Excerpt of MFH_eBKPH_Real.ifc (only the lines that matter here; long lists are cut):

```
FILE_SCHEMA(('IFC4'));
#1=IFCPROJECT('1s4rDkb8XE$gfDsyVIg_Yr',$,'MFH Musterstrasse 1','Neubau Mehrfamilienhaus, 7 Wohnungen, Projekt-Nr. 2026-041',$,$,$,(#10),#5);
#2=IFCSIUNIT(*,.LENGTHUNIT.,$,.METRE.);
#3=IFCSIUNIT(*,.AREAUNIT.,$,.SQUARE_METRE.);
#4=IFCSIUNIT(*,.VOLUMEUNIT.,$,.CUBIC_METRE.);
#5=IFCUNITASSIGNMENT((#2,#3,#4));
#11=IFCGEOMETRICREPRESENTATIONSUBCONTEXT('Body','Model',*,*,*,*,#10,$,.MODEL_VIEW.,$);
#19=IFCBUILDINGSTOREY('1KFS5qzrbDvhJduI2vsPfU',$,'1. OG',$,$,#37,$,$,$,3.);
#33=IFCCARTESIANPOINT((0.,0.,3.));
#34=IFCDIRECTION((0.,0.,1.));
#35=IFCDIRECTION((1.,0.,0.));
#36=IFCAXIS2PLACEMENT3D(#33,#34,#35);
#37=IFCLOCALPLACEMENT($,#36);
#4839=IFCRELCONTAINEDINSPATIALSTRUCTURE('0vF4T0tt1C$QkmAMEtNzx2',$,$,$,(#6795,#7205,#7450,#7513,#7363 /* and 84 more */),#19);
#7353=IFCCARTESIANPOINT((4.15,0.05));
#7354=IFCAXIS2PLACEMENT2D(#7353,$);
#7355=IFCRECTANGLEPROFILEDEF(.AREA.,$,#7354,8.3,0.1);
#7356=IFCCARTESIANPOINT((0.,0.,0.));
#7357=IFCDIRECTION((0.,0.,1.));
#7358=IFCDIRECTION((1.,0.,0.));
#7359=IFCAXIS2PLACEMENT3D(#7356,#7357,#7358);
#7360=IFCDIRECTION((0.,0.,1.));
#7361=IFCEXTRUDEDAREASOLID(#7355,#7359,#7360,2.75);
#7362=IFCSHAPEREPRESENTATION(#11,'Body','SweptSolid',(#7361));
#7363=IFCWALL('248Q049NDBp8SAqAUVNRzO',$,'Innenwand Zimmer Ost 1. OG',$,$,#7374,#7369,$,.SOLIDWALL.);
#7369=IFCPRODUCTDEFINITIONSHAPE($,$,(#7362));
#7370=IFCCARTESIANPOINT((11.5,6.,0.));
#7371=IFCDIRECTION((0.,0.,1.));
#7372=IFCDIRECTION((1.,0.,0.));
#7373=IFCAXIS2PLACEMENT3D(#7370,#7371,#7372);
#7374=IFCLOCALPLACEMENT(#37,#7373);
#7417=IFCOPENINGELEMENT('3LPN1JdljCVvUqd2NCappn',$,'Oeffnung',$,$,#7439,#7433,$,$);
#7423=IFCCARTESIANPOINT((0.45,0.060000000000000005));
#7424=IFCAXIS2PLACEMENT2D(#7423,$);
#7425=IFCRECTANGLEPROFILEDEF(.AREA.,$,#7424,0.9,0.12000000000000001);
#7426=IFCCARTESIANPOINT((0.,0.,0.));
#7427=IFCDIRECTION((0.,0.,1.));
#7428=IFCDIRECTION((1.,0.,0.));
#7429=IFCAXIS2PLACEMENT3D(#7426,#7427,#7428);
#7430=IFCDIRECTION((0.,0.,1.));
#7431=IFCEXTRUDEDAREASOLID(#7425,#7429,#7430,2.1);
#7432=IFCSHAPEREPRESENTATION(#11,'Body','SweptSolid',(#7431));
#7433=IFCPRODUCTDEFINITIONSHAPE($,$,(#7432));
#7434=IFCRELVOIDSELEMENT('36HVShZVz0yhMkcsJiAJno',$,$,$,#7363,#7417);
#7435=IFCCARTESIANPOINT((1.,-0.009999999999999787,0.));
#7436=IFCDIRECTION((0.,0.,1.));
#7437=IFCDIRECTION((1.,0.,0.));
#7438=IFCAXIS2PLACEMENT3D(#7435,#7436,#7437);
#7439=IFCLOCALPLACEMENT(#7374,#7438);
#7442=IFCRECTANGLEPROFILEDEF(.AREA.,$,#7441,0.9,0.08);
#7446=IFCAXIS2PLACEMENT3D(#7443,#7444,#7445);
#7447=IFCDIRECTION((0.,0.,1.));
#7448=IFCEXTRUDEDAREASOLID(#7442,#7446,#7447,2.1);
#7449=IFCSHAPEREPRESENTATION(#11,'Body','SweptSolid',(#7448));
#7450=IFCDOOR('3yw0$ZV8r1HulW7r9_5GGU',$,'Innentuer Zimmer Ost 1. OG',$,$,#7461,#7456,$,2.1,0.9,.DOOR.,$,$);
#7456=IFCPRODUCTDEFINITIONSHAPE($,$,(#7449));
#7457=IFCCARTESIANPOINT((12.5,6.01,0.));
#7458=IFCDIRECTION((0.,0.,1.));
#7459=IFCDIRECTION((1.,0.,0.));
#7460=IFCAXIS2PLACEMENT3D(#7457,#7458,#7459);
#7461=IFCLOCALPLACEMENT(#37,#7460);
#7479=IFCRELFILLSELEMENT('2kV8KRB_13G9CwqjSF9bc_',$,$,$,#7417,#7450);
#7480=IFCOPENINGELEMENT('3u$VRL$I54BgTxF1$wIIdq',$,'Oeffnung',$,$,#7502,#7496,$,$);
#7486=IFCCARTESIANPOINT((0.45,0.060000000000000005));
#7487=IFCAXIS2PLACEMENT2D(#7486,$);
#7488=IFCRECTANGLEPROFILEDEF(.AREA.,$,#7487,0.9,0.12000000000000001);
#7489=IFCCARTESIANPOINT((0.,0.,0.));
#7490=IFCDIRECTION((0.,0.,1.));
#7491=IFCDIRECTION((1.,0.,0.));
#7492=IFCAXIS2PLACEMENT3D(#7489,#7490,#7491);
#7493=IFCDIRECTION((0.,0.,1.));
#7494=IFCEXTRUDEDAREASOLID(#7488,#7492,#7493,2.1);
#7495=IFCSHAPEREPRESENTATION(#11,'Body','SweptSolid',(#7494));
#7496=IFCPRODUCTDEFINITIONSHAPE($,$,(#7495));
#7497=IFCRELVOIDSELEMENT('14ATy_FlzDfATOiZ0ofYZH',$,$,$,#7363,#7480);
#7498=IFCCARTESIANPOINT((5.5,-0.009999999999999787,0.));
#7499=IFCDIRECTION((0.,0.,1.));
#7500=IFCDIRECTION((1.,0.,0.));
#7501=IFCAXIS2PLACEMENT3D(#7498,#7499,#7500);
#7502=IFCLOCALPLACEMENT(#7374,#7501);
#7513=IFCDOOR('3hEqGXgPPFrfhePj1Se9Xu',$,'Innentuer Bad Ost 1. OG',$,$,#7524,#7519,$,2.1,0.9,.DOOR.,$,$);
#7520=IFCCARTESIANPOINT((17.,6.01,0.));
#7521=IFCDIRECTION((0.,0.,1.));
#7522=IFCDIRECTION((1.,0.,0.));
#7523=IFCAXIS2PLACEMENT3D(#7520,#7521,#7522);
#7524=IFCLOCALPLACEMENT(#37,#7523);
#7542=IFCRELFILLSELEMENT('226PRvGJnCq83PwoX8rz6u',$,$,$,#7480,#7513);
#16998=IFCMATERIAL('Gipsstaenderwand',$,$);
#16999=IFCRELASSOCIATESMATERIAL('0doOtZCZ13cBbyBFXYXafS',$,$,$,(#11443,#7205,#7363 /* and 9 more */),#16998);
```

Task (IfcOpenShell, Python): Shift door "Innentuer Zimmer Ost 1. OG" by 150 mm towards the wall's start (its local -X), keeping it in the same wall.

```python
import ifcopenshell
import ifcopenshell.api.geometry
import ifcopenshell.util.placement

model = ifcopenshell.open("MFH_eBKPH_Real.ifc")

door = model.by_guid("3yw0$ZV8r1HulW7r9_5GGU")
opening = door.FillsVoids[0].RelatingOpeningElement
wall = opening.VoidsElements[0].RelatingBuildingElement

wall_matrix = ifcopenshell.util.placement.get_local_placement(wall.ObjectPlacement)
shift = wall_matrix[:3, 0] * -0.15
before = ifcopenshell.util.placement.get_local_placement(door.ObjectPlacement)[:3, 3].copy()

# The door is not placed relative to its opening, so move both.
for product in (opening, door):
    matrix = ifcopenshell.util.placement.get_local_placement(product.ObjectPlacement)
    matrix[:3, 3] += shift
    ifcopenshell.api.geometry.edit_object_placement(model, product=product, matrix=matrix, is_si=False)

after = ifcopenshell.util.placement.get_local_placement(door.ObjectPlacement)[:3, 3]
print("door moved by", (after - before).round(3) + 0.0)

model.write("MFH_eBKPH_Real_edited.ifc")
```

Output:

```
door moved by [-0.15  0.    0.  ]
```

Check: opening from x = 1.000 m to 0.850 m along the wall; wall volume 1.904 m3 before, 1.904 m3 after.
